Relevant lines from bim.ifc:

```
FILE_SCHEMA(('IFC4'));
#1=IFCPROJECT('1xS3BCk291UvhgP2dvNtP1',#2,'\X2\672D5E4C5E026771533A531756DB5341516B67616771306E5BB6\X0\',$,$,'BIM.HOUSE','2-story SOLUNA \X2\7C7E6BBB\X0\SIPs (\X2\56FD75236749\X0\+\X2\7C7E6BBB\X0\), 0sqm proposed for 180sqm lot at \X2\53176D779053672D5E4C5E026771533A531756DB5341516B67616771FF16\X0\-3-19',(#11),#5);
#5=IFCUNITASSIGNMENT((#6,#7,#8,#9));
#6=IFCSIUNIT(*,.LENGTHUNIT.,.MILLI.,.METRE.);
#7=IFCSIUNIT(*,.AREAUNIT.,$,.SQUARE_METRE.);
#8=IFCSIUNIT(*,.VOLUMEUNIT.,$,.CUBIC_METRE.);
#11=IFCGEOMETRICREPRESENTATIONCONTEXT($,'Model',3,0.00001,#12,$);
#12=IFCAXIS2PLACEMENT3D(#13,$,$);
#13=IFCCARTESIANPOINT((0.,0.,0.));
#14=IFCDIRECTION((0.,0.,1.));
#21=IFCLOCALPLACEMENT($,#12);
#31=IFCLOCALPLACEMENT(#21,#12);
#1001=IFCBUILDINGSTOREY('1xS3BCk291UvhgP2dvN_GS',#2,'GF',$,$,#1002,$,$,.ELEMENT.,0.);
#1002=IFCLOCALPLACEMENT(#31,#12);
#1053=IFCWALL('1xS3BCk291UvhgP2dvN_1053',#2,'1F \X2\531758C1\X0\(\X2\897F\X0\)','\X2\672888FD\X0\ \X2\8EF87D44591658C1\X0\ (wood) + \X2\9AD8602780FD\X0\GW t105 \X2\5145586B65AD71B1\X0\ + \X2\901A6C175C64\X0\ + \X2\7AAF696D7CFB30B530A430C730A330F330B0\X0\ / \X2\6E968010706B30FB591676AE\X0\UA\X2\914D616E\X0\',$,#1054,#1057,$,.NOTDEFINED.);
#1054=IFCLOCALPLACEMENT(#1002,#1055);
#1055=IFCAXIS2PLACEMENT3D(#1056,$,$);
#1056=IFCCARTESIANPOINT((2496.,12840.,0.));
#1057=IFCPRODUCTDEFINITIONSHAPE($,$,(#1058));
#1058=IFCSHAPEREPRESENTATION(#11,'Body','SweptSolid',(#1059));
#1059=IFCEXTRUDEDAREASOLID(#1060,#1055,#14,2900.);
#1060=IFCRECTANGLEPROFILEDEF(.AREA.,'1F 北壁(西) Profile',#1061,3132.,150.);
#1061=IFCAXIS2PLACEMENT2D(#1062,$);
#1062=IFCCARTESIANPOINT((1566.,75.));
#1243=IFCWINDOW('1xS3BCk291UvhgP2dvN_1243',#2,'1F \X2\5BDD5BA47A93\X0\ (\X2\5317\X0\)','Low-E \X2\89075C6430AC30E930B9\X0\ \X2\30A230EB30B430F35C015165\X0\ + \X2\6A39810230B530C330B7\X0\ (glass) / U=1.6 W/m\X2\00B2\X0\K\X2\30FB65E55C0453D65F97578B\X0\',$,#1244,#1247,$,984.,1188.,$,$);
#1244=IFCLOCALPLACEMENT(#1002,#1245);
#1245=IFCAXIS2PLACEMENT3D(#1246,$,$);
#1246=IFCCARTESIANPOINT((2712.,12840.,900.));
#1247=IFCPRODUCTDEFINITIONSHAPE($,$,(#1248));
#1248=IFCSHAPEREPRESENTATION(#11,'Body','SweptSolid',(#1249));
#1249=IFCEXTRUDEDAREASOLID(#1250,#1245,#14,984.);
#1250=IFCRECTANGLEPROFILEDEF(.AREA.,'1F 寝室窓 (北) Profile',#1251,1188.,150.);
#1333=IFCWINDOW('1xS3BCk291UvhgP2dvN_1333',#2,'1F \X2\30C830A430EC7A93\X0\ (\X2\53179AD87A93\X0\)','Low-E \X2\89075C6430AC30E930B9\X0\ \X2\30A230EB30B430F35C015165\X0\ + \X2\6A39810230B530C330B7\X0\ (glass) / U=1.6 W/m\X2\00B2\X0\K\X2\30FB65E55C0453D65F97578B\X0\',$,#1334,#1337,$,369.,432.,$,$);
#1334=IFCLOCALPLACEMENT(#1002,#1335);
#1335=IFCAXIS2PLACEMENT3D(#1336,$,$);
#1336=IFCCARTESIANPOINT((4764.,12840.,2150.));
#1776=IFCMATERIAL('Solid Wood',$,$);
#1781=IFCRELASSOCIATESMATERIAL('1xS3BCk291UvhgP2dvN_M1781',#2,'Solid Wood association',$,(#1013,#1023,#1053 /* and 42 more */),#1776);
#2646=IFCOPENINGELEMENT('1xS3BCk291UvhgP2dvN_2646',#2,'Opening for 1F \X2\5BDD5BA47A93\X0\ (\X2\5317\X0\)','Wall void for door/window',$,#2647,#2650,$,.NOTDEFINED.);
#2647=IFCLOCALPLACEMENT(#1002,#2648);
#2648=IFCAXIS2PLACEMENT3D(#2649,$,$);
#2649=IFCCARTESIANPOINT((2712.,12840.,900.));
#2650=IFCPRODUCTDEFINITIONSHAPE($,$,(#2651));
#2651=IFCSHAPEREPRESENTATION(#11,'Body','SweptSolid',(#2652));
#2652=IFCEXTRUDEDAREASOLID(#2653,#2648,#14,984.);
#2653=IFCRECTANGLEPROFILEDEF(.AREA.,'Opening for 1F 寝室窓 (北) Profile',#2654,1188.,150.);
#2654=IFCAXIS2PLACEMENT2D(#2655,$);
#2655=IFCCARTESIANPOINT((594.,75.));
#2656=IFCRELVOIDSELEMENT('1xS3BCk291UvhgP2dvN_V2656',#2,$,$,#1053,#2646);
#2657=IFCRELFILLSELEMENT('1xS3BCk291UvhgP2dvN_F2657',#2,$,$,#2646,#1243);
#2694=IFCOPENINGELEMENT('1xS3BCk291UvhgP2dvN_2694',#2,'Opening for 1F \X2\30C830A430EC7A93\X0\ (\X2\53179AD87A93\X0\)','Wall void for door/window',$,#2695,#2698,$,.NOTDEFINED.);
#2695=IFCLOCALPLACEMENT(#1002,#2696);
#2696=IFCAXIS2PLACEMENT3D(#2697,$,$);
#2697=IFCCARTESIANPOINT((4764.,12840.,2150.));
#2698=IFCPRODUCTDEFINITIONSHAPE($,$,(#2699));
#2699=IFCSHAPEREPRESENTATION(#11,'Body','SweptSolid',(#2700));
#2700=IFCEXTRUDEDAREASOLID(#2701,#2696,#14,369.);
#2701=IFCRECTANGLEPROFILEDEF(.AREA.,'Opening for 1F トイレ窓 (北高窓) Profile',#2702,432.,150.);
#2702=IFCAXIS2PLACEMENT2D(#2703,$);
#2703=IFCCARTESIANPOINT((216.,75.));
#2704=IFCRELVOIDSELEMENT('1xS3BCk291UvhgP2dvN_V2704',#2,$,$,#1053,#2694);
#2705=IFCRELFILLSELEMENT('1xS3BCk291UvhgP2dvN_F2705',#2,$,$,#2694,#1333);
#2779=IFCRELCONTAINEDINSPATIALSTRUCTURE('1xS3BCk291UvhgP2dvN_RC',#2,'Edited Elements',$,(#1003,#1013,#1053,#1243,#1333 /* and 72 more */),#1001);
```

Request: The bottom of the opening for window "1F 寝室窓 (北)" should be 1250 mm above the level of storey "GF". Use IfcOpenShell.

```python
import numpy as np
import ifcopenshell
import ifcopenshell.api.geometry
import ifcopenshell.geom
import ifcopenshell.util.element
import ifcopenshell.util.placement
import ifcopenshell.util.shape
import ifcopenshell.util.unit

model = ifcopenshell.open("bim.ifc")
unit_scale = ifcopenshell.util.unit.calculate_unit_scale(model)

window = model.by_guid("1xS3BCk291UvhgP2dvN_1243")
opening = window.FillsVoids[0].RelatingOpeningElement
storey = ifcopenshell.util.element.get_container(window, ifc_class="IfcBuildingStorey")
level = ifcopenshell.util.placement.get_local_placement(storey.ObjectPlacement)[2, 3]

# The opening's origin need not be at the sill, so measure its lowest point.
shape = ifcopenshell.geom.create_shape(ifcopenshell.geom.settings(), opening)
bottom = ifcopenshell.util.shape.get_shape_bottom_elevation(shape, shape.geometry) / unit_scale
dz = level + 1250.0 - bottom

shift = np.array([0.0, 0.0, dz])
# The window is not placed relative to its opening, so move both.
for product in (opening, window):
    matrix = ifcopenshell.util.placement.get_local_placement(product.ObjectPlacement)
    matrix[:3, 3] += shift
    ifcopenshell.api.geometry.edit_object_placement(model, product=product, matrix=matrix, is_si=False)

print(f"moved by {dz * unit_scale:+.3f} m")

model.write("bim_rev.ifc")
```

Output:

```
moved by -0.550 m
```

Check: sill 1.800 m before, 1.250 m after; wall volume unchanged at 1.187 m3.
